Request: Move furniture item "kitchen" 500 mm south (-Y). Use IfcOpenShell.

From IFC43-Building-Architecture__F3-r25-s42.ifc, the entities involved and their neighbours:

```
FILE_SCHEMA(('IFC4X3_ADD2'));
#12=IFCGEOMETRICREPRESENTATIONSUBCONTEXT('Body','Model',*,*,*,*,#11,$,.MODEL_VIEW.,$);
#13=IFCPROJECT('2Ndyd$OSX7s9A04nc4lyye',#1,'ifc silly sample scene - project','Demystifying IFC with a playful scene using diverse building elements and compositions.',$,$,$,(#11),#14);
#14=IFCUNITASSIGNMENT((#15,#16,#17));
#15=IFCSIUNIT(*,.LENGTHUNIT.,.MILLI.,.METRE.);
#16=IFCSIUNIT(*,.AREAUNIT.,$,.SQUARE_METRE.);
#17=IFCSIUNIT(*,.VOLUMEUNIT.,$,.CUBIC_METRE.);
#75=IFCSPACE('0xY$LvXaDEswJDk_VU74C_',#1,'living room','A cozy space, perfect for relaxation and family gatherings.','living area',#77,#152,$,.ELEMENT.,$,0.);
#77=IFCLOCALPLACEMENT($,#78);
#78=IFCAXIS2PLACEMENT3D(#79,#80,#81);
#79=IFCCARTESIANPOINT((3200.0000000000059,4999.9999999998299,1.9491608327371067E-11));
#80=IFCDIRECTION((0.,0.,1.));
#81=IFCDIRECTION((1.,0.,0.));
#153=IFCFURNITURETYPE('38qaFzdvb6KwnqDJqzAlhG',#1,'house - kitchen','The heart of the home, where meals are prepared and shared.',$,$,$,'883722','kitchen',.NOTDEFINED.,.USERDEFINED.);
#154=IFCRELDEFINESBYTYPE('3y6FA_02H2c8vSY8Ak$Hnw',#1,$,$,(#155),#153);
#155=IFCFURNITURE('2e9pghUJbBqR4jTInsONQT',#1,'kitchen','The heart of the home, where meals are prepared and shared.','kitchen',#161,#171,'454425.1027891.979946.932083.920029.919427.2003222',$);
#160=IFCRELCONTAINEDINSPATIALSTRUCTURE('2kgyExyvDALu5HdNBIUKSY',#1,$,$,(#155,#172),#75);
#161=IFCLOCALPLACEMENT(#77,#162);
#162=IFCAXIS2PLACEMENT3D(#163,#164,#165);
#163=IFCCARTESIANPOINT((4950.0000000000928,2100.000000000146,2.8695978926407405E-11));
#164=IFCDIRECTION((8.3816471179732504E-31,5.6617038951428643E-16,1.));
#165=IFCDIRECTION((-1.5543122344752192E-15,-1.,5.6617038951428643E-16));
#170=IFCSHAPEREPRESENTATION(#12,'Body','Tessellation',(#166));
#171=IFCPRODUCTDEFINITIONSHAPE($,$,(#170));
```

```python
import ifcopenshell
import ifcopenshell.api.geometry
import ifcopenshell.util.placement
import ifcopenshell.util.unit

model = ifcopenshell.open("IFC43-Building-Architecture__F3-r25-s42.ifc")
unit_scale = ifcopenshell.util.unit.calculate_unit_scale(model)

item = model.by_guid("2e9pghUJbBqR4jTInsONQT")
matrix = ifcopenshell.util.placement.get_local_placement(item.ObjectPlacement)
matrix[1, 3] -= 0.5 / unit_scale
ifcopenshell.api.geometry.edit_object_placement(model, product=item, matrix=matrix, is_si=False)

print(ifcopenshell.util.placement.get_local_placement(item.ObjectPlacement).round(3) + 0.0)

model.write("IFC43-Building-Architecture__F3-r25-s42_updated.ifc")
```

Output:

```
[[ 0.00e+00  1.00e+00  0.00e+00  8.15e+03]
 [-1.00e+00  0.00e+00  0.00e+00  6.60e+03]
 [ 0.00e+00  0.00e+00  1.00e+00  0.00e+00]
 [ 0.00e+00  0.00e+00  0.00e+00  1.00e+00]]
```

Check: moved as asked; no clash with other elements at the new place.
